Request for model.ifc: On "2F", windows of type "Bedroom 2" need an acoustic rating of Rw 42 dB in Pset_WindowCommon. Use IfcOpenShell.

First a look at what the model holds.

```python
import ifcopenshell
import ifcopenshell.util.element

model = ifcopenshell.open("model.ifc")
print(model.schema)
storey = next(s for s in model.by_type("IfcBuildingStorey") if s.Name == "2F")
windows = [e for e in ifcopenshell.util.element.get_decomposition(storey) if e.is_a("IfcWindow")]
seen = {}
for e in windows:
    element_type = ifcopenshell.util.element.get_type(e)
    key = (element_type.Name if element_type != e and element_type else None, ifcopenshell.util.element.get_pset(e, "Pset_WindowCommon", "AcousticRating"))
    seen[key] = seen.get(key, 0) + 1
for (name, value), count in sorted(seen.items(), key=str):
    print(count, "x", name, "|", value)
```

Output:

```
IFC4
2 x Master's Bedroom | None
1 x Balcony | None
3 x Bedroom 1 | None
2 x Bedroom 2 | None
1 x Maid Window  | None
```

```python
import ifcopenshell
import ifcopenshell.api.pset
import ifcopenshell.util.element

model = ifcopenshell.open("model.ifc")

storey = next(s for s in model.by_type("IfcBuildingStorey") if s.Name == "2F")
windows = [e for e in ifcopenshell.util.element.get_decomposition(storey) if e.is_a("IfcWindow")]

count = 0
for e in windows:
    element_type = ifcopenshell.util.element.get_type(e)
    if element_type in (None, e) or element_type.Name != "Bedroom 2":
        continue
    # add_pset returns the element's existing set when there is one.
    pset = ifcopenshell.api.pset.add_pset(model, product=e, name="Pset_WindowCommon")
    ifcopenshell.api.pset.edit_pset(model, pset=pset, properties={"AcousticRating": "Rw 42 dB"})
    count += 1

print(count, "windows updated")

model.write("model_rev.ifc")
```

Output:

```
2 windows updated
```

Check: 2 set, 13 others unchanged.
